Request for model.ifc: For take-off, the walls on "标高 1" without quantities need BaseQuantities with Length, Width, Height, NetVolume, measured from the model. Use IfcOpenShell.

First a look at what the model holds.

```python
import ifcopenshell
import ifcopenshell.util.element
import ifcopenshell.util.unit

model = ifcopenshell.open("model.ifc")
print(model.schema)
for unit_type in ("LENGTHUNIT", "AREAUNIT", "VOLUMEUNIT"):
    print(unit_type, ifcopenshell.util.unit.calculate_unit_scale(model, unit_type))
storey = next(s for s in model.by_type("IfcBuildingStorey") if s.Name == "标高 1")
walls = [e for e in ifcopenshell.util.element.get_decomposition(storey) if e.is_a("IfcWall")]
for e in sorted(walls, key=lambda e: e.id()):
    print(e.id(), e.is_a(), e.Name, list(ifcopenshell.util.element.get_psets(e, qtos_only=True)), sep=" | ")
```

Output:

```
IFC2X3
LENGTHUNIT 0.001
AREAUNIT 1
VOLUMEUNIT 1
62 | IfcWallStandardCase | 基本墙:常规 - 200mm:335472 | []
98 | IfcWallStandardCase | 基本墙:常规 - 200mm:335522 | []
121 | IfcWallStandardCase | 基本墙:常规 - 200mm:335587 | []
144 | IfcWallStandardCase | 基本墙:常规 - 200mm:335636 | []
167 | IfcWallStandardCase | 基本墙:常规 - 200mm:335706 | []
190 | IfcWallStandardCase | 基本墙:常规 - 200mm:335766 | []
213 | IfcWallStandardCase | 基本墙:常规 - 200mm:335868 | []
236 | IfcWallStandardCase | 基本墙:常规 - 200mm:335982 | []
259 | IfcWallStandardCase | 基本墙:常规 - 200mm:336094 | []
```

```python
import ifcopenshell
import ifcopenshell.api.pset
import ifcopenshell.geom
import ifcopenshell.util.element
import ifcopenshell.util.shape
import ifcopenshell.util.unit

model = ifcopenshell.open("model.ifc")
unit_scale = ifcopenshell.util.unit.calculate_unit_scale(model)
volume_scale = ifcopenshell.util.unit.calculate_unit_scale(model, "VOLUMEUNIT")
settings = ifcopenshell.geom.settings()

storey = next(s for s in model.by_type("IfcBuildingStorey") if s.Name == "标高 1")
walls = [e for e in ifcopenshell.util.element.get_decomposition(storey) if e.is_a("IfcWall")]

for e in sorted(walls, key=lambda e: e.id()):
    if ifcopenshell.util.element.get_psets(e, qtos_only=True, should_inherit=False):
        continue
    # Geometry comes back in metres, in the element's own axes.
    shape = ifcopenshell.geom.create_shape(settings, e)
    values = {
        "Length": ifcopenshell.util.shape.get_x(shape.geometry) / unit_scale,
        "Width": ifcopenshell.util.shape.get_y(shape.geometry) / unit_scale,
        "Height": ifcopenshell.util.shape.get_z(shape.geometry) / unit_scale,
        "NetVolume": ifcopenshell.util.shape.get_volume(shape.geometry) / volume_scale,
    }
    qto = ifcopenshell.api.pset.add_qto(model, product=e, name="BaseQuantities")
    ifcopenshell.api.pset.edit_qto(model, qto=qto, properties=values)
    print(e.id(), {k: round(v, 3) for k, v in values.items()})

model.write("model_edited.ifc")
```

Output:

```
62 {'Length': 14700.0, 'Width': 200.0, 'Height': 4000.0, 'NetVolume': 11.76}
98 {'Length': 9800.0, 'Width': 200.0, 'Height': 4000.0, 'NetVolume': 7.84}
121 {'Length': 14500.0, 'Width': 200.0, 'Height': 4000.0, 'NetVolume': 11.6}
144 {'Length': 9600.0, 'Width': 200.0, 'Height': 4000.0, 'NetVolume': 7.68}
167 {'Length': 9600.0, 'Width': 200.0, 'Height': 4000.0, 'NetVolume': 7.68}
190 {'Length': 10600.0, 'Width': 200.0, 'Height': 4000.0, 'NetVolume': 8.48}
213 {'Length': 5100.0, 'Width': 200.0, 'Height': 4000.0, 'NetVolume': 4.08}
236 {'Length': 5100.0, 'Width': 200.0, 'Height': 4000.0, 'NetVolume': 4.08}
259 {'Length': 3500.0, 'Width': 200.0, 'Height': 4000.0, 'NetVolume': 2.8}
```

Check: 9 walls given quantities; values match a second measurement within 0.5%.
